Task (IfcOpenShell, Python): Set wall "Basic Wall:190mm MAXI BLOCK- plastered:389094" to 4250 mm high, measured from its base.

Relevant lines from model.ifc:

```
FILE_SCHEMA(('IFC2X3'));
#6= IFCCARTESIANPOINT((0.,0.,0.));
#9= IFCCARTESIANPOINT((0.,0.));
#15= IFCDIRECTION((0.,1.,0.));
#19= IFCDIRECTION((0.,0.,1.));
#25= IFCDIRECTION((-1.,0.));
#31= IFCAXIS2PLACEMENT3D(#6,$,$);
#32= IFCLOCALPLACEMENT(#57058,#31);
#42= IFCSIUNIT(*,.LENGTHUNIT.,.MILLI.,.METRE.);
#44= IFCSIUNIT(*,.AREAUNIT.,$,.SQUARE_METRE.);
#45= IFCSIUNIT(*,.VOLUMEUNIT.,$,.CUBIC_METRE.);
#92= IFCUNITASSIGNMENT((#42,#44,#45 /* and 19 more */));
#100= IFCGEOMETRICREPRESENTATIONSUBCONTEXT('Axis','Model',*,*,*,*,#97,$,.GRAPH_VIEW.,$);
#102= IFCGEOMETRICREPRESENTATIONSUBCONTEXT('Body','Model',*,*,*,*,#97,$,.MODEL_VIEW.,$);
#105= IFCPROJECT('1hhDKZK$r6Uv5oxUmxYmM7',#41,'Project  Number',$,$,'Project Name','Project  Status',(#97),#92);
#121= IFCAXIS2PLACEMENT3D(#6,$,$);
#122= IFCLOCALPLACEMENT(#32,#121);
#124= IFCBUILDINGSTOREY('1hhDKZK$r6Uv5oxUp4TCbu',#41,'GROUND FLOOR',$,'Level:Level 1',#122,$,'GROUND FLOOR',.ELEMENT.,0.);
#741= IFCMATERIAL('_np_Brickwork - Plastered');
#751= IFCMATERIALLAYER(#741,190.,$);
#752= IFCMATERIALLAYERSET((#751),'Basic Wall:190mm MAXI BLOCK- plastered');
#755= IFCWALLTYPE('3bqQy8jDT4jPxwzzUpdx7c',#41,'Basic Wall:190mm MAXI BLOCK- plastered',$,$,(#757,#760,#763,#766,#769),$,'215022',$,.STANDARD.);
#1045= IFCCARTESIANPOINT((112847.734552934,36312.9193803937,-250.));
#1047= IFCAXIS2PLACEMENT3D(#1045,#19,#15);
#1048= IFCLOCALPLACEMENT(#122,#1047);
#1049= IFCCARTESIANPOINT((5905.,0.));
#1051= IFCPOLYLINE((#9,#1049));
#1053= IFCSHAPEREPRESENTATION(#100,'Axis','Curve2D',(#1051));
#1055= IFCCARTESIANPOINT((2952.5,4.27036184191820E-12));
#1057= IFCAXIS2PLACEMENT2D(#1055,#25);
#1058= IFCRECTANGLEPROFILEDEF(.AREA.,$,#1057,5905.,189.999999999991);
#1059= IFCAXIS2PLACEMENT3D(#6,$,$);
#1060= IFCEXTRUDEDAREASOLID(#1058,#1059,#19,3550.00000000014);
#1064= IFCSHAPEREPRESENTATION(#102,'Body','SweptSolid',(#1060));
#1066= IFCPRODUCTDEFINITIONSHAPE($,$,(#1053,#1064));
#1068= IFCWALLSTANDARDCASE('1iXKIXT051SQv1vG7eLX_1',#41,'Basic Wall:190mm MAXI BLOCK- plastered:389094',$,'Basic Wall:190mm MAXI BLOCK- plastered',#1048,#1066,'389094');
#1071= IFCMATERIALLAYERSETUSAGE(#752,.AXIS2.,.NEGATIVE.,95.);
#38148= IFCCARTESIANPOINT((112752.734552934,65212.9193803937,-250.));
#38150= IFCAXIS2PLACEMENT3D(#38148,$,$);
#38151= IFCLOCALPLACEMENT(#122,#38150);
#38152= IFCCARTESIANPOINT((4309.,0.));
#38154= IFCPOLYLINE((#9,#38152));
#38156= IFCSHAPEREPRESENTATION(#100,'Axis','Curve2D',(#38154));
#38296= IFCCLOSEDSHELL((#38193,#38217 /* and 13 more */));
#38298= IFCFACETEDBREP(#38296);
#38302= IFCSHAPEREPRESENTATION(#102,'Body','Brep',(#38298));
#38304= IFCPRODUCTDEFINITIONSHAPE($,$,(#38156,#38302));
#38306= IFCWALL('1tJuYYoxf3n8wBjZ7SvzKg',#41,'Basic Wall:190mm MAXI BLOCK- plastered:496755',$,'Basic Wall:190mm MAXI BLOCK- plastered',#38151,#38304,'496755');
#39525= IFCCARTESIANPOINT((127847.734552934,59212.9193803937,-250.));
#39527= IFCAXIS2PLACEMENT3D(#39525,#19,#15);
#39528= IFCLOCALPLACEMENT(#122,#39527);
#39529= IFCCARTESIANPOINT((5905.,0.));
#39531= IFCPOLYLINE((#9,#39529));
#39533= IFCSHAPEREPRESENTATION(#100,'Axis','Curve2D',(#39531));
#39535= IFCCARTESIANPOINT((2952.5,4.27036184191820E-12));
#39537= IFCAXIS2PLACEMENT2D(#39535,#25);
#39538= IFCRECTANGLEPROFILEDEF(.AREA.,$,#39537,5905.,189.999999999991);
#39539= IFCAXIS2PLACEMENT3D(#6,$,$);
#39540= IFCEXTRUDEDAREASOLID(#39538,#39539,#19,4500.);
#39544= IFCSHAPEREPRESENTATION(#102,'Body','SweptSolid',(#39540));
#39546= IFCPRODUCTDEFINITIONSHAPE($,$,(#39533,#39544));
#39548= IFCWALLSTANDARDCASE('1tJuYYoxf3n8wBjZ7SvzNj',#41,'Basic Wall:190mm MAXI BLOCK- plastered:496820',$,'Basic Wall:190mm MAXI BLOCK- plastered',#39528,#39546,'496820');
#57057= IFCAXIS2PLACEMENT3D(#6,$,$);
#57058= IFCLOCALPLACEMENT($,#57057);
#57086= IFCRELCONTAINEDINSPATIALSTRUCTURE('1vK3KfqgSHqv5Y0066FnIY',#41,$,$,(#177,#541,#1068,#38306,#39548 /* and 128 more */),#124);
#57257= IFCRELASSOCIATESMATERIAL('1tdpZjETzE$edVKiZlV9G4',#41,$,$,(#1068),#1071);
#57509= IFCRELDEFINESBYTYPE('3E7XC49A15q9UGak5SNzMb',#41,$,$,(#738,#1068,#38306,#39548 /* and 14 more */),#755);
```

```python
import ifcopenshell
import ifcopenshell.geom
import ifcopenshell.util.representation
import ifcopenshell.util.shape

model = ifcopenshell.open("model.ifc")
settings = ifcopenshell.geom.settings()


def volume(element):
    """Net volume in cubic metres, openings subtracted."""
    shape = ifcopenshell.geom.create_shape(settings, element)
    return ifcopenshell.util.shape.get_volume(shape.geometry)


wall = model.by_guid("1iXKIXT051SQv1vG7eLX_1")
before = volume(wall)

body = ifcopenshell.util.representation.get_representation(wall, "Model", "Body")
solid = body.Items[0]
old_height = solid.Depth
solid.Depth = 4250.0
after = volume(wall)

print(f"height {old_height:g} -> {solid.Depth:g}, volume {before:.3f} -> {after:.3f} m3")

model.write("model-out.ifc")
```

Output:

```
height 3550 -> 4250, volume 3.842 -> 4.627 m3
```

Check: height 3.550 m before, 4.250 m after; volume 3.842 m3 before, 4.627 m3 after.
